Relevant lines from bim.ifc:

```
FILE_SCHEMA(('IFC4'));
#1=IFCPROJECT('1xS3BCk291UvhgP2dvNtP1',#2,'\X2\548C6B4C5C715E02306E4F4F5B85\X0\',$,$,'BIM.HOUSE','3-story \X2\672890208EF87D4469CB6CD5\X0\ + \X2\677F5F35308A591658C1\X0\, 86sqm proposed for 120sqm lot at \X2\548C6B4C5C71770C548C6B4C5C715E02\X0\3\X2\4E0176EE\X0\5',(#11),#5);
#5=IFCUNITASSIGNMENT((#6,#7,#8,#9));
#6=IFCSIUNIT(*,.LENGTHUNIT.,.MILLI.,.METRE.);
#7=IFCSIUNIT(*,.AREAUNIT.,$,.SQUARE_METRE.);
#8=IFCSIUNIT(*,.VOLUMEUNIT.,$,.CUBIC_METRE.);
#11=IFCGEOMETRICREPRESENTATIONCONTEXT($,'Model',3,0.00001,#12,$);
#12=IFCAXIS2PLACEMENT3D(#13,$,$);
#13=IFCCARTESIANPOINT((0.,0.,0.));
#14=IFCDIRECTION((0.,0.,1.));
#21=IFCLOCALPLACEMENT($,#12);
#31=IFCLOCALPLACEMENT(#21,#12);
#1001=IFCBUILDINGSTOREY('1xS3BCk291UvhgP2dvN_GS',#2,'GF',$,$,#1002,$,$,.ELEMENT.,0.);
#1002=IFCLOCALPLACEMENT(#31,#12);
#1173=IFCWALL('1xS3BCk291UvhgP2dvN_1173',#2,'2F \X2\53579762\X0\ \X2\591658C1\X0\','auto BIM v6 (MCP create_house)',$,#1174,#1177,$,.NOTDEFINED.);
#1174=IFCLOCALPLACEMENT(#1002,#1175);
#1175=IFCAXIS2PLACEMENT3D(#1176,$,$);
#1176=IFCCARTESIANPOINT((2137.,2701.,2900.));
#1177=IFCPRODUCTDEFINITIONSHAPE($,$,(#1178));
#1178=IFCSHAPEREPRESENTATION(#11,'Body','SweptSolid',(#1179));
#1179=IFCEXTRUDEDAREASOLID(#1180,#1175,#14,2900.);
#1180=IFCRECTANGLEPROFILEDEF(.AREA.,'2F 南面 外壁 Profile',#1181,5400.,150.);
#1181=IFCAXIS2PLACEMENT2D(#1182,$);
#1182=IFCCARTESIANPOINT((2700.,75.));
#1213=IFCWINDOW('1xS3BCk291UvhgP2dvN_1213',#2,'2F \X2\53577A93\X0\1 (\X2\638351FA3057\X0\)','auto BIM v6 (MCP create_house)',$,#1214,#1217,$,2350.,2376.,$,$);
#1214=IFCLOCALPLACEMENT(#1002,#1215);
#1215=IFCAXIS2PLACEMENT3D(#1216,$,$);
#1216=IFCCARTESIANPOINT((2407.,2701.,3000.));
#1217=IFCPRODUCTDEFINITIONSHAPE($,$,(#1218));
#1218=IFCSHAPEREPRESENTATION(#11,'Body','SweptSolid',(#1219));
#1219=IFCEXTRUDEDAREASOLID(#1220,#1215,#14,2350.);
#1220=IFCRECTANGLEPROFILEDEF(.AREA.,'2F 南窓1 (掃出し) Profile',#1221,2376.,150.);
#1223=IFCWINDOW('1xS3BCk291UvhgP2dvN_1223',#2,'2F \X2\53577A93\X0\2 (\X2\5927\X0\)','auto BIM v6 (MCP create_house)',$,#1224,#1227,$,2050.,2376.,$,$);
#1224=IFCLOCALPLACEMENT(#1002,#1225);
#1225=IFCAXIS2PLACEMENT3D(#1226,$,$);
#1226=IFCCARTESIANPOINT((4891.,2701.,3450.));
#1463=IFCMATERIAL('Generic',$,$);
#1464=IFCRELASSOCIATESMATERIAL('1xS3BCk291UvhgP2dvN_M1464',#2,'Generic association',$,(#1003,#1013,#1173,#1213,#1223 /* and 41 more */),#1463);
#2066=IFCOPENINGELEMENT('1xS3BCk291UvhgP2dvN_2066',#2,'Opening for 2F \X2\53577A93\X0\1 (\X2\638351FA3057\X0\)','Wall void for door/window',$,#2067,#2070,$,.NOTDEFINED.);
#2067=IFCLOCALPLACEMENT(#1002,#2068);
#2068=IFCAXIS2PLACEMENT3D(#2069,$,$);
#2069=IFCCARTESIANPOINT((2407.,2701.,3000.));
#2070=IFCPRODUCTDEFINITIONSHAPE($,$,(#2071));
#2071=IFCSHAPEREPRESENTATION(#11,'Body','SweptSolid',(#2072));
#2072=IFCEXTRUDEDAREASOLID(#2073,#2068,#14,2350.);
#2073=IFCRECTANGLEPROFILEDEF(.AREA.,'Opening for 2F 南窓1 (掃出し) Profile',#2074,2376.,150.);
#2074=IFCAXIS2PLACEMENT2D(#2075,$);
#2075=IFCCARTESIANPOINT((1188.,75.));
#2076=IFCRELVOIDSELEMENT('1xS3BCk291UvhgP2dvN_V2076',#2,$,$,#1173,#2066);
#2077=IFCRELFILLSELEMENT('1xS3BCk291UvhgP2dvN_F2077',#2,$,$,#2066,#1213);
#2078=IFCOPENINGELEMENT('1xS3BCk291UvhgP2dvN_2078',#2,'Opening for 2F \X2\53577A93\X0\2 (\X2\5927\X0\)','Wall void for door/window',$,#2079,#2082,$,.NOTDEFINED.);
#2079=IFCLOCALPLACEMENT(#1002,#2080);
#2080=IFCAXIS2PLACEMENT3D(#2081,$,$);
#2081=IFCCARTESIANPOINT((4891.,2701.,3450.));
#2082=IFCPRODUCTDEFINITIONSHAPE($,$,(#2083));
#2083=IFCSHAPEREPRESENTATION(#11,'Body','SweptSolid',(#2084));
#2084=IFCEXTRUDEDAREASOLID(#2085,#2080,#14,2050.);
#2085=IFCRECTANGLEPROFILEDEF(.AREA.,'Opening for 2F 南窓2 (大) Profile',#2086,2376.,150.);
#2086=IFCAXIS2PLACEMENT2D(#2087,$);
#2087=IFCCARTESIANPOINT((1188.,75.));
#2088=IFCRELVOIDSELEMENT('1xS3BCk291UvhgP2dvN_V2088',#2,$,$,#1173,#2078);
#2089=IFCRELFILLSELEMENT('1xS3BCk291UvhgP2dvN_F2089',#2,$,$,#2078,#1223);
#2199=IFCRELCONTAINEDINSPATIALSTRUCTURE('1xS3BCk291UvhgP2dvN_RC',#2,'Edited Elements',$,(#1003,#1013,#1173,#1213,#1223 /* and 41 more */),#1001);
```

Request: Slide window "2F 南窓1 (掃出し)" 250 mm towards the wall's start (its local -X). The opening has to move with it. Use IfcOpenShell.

```python
import ifcopenshell
import ifcopenshell.api.geometry
import ifcopenshell.util.placement

model = ifcopenshell.open("bim.ifc")

window = model.by_guid("1xS3BCk291UvhgP2dvN_1213")
opening = window.FillsVoids[0].RelatingOpeningElement
wall = opening.VoidsElements[0].RelatingBuildingElement

wall_matrix = ifcopenshell.util.placement.get_local_placement(wall.ObjectPlacement)
shift = wall_matrix[:3, 0] * -250.0
before = ifcopenshell.util.placement.get_local_placement(window.ObjectPlacement)[:3, 3].copy()

# The window is not placed relative to its opening, so move both.
for product in (opening, window):
    matrix = ifcopenshell.util.placement.get_local_placement(product.ObjectPlacement)
    matrix[:3, 3] += shift
    ifcopenshell.api.geometry.edit_object_placement(model, product=product, matrix=matrix, is_si=False)

after = ifcopenshell.util.placement.get_local_placement(window.ObjectPlacement)[:3, 3]
print("window moved by", (after - before).round(3) + 0.0)

model.write("bim-out.ifc")
```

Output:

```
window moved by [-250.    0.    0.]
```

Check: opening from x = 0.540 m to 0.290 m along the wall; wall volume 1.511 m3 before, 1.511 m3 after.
